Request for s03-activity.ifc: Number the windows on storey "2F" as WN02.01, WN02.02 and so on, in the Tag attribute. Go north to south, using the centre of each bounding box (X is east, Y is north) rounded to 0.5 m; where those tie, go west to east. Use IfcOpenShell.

First a look at what the model holds.

```python
import ifcopenshell
import ifcopenshell.util.element
import ifcopenshell.util.placement

model = ifcopenshell.open("s03-activity.ifc")
print(model.schema)
storey = next(s for s in model.by_type("IfcBuildingStorey") if s.Name == "2F")
windows = [e for e in ifcopenshell.util.element.get_decomposition(storey) if e.is_a("IfcWindow")]
for e in sorted(windows, key=lambda e: e.id()):
    origin = ifcopenshell.util.placement.get_local_placement(e.ObjectPlacement)[:3, 3]
    print(e.id(), e.Tag, e.Name, origin.round(2) + 0.0, sep=" | ")
```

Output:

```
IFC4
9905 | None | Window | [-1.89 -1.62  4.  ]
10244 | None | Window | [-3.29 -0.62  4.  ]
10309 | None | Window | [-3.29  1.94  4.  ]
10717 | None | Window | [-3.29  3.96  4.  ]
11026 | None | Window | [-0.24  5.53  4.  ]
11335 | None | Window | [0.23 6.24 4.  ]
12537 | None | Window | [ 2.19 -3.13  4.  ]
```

```python
import ifcopenshell
import ifcopenshell.geom
import ifcopenshell.util.element
import ifcopenshell.util.shape

model = ifcopenshell.open("s03-activity.ifc")
settings = ifcopenshell.geom.settings()
settings.set("use-world-coords", True)


def centre(element):
    shape = ifcopenshell.geom.create_shape(settings, element)
    return ifcopenshell.util.shape.get_bbox_centroid(shape.geometry)


storey = next(s for s in model.by_type("IfcBuildingStorey") if s.Name == "2F")
windows = [e for e in ifcopenshell.util.element.get_decomposition(storey) if e.is_a("IfcWindow")]

# Insertion points can sit at a corner or the storey origin, so sort by the geometry (in metres).
centres = {e: centre(e) for e in windows}
windows.sort(key=lambda e: (-round(centres[e][1] / 0.5), centres[e][0]))

for i, e in enumerate(windows, start=1):
    number = f"WN02.{i:02d}"
    e.Tag = number
    print(e.id(), number)

model.write("s03-activity_rev.ifc")
```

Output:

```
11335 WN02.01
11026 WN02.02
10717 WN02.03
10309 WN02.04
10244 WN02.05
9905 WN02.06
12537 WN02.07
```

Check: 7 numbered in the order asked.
